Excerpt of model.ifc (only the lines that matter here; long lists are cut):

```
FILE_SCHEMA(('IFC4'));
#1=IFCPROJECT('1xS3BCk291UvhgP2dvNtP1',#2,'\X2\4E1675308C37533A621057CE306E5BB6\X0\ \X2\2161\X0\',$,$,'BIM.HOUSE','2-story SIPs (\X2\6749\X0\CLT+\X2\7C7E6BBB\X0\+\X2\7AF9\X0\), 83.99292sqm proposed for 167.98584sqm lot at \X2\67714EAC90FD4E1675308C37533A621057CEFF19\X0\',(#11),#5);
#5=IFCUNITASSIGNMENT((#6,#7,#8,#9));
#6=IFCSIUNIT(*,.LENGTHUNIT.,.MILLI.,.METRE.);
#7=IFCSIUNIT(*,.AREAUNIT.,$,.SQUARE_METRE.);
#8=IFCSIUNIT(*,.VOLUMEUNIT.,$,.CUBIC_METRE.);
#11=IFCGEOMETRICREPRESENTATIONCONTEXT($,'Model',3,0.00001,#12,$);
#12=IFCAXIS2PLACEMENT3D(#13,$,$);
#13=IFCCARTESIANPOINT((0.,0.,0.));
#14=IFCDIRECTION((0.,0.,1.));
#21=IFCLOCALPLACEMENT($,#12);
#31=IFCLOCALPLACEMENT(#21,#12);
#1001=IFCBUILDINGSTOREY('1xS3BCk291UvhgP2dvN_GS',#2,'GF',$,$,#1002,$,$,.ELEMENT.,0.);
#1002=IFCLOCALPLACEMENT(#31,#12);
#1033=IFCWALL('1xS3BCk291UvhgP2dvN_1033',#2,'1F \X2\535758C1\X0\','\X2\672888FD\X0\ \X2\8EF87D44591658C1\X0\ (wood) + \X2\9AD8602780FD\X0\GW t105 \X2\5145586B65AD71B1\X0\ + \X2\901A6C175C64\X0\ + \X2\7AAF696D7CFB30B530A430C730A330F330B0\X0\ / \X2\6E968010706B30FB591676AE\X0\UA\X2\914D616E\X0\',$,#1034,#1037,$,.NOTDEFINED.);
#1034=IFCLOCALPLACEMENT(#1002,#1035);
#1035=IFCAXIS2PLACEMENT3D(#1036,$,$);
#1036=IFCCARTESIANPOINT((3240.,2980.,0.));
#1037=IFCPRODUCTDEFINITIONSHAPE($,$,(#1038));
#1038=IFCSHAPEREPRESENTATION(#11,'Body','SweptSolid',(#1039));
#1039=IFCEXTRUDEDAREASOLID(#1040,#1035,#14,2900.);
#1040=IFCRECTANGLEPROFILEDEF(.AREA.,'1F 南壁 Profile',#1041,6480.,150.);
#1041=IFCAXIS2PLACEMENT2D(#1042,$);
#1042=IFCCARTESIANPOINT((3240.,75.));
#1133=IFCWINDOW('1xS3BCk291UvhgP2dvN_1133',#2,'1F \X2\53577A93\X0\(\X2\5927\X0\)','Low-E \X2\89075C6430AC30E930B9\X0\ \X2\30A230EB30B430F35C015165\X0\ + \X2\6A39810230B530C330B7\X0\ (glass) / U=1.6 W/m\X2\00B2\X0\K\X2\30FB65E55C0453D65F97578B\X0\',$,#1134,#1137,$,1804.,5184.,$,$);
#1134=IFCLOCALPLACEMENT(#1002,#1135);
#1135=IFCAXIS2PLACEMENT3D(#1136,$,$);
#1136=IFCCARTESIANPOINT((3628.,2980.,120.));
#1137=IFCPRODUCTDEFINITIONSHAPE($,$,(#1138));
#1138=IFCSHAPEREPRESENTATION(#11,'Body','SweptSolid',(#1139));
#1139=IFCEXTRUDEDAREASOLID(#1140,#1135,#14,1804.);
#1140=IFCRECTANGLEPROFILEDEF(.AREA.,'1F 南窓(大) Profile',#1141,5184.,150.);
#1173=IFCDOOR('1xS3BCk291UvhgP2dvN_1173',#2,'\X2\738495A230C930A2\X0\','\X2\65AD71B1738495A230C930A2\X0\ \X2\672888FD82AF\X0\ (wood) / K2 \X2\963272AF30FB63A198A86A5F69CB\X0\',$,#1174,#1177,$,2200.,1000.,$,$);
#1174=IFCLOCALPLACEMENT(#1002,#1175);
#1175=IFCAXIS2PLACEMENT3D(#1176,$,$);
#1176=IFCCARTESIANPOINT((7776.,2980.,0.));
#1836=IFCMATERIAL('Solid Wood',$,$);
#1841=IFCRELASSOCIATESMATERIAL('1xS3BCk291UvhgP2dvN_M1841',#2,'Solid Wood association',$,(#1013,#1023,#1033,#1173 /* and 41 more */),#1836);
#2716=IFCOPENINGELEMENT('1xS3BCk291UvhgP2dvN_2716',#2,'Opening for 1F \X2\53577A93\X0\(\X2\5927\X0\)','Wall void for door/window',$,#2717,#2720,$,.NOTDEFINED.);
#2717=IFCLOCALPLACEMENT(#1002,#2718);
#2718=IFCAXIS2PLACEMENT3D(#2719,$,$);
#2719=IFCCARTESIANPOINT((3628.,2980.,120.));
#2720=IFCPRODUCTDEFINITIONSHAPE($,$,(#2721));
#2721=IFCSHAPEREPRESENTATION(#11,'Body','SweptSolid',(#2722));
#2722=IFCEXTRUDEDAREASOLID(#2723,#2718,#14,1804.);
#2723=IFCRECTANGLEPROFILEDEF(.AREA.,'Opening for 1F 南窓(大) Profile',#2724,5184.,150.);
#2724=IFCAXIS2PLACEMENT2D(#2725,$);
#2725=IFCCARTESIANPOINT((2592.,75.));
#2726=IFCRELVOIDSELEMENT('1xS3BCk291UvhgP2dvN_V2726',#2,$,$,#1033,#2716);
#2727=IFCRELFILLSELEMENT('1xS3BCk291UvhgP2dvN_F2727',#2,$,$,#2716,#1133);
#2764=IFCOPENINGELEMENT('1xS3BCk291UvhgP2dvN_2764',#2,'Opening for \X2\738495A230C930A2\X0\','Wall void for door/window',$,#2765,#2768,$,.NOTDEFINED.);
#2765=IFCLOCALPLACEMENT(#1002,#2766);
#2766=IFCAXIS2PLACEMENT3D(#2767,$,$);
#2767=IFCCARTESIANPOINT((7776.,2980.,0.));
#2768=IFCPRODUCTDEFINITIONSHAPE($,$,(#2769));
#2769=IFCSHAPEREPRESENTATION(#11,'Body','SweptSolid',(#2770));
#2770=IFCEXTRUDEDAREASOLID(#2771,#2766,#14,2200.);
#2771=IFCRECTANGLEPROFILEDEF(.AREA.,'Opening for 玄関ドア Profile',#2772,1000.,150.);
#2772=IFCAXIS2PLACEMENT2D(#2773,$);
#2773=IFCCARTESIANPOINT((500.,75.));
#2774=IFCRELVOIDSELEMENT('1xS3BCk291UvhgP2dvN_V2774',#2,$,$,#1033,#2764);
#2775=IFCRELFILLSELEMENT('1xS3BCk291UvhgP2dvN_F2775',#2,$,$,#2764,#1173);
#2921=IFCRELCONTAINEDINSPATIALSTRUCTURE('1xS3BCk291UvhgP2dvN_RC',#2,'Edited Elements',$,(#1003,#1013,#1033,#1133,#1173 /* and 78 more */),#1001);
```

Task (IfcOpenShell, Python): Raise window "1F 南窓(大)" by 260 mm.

```python
import numpy as np
import ifcopenshell
import ifcopenshell.api.geometry
import ifcopenshell.util.placement
import ifcopenshell.util.unit

model = ifcopenshell.open("model.ifc")
unit_scale = ifcopenshell.util.unit.calculate_unit_scale(model)

window = model.by_guid("1xS3BCk291UvhgP2dvN_1133")
opening = window.FillsVoids[0].RelatingOpeningElement
dz = 260.0

shift = np.array([0.0, 0.0, dz])
# The window is not placed relative to its opening, so move both.
for product in (opening, window):
    matrix = ifcopenshell.util.placement.get_local_placement(product.ObjectPlacement)
    matrix[:3, 3] += shift
    ifcopenshell.api.geometry.edit_object_placement(model, product=product, matrix=matrix, is_si=False)

print(f"moved by {dz * unit_scale:+.3f} m")

model.write("model_updated.ifc")
```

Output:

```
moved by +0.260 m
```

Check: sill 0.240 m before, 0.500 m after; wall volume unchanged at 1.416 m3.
